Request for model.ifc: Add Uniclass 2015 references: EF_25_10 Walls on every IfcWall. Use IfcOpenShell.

First a look at what the model holds.

```python
import ifcopenshell

model = ifcopenshell.open("model.ifc")
print(model.schema)
print("classifications:", [c.Name for c in model.by_type("IfcClassification")])
for ifc_class in ("IfcDoor", "IfcRoof", "IfcStair", "IfcWall", "IfcWindow"):
    print(ifc_class, len(model.by_type(ifc_class)))
```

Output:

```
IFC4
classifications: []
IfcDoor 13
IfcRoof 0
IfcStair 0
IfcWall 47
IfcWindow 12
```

```python
import ifcopenshell
import ifcopenshell.api.classification

model = ifcopenshell.open("model.ifc")

system = ifcopenshell.api.classification.add_classification(model, classification="Uniclass 2015")

codes = {
    "IfcWall": ("EF_25_10", "Walls"),
}
for ifc_class, (code, name) in codes.items():
    products = model.by_type(ifc_class)
    ifcopenshell.api.classification.add_reference(
        model, products=products, classification=system, identification=code, name=name
    )
    print(code, len(products))

model.write("model-out.ifc")
```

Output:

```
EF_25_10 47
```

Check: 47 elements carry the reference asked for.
